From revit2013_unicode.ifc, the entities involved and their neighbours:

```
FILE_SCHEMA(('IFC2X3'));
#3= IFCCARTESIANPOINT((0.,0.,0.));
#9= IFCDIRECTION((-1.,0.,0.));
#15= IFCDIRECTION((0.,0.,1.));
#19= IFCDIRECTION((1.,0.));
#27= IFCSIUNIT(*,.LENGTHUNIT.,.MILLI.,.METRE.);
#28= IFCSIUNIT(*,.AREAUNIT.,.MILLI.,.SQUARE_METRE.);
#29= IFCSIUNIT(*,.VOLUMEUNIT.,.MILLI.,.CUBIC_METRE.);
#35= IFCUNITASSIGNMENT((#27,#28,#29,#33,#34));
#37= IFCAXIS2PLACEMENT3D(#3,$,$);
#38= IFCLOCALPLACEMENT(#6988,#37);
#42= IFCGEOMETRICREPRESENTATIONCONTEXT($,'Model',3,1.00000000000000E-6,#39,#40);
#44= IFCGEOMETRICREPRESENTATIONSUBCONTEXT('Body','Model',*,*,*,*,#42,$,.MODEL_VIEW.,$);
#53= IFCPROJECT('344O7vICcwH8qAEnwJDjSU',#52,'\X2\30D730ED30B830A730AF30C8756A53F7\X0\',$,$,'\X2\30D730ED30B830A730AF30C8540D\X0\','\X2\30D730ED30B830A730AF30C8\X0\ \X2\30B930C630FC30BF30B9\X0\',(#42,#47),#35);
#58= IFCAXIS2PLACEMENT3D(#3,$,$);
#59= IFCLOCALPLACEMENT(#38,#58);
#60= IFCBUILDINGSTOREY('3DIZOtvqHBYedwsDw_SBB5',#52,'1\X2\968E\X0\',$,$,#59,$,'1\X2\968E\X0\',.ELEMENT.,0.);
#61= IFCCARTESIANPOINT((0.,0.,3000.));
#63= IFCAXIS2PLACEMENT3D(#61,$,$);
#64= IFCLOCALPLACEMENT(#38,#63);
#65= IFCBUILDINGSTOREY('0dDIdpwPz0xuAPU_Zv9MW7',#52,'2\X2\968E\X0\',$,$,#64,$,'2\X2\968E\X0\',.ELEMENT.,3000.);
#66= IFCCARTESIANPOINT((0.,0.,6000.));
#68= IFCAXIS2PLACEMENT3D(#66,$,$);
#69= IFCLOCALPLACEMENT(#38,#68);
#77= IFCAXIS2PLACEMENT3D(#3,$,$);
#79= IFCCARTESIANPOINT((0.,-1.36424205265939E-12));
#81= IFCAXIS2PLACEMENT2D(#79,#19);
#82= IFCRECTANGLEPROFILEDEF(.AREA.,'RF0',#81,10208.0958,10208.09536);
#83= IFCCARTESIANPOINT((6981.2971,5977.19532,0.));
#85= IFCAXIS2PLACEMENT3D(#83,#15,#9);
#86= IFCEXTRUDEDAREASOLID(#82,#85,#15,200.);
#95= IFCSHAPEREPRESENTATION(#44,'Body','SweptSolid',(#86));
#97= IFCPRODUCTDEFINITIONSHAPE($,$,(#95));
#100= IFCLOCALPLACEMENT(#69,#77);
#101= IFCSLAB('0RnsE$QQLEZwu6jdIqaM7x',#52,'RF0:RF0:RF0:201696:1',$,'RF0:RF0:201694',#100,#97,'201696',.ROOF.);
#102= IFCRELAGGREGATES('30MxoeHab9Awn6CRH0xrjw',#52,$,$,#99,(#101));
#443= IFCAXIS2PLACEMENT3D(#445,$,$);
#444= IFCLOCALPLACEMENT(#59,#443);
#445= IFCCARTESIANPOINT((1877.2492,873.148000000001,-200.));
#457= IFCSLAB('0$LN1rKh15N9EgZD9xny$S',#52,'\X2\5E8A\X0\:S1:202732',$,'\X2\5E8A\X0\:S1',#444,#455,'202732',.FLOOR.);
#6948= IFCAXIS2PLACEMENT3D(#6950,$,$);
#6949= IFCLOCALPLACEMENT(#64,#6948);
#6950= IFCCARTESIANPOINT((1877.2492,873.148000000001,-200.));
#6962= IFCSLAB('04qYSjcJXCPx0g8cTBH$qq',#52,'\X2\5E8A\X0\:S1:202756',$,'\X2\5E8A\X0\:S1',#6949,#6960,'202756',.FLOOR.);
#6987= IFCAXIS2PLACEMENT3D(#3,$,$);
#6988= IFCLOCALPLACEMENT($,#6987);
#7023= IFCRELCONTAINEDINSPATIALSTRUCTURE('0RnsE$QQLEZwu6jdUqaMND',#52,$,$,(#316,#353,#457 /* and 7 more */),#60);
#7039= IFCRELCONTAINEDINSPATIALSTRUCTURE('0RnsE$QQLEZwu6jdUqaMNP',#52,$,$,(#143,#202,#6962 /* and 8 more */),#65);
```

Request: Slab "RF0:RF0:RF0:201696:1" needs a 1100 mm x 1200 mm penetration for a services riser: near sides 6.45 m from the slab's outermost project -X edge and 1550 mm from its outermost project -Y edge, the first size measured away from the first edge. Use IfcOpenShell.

```python
import numpy as np
import ifcopenshell
import ifcopenshell.api.feature
import ifcopenshell.api.geometry
import ifcopenshell.api.root
import ifcopenshell.geom
import ifcopenshell.util.placement
import ifcopenshell.util.representation
import ifcopenshell.util.shape
import ifcopenshell.util.unit

model = ifcopenshell.open("revit2013_unicode.ifc")
unit_scale = ifcopenshell.util.unit.calculate_unit_scale(model)
settings = ifcopenshell.geom.settings()


def volume(element):
    """Net volume in cubic metres, openings subtracted."""
    shape = ifcopenshell.geom.create_shape(settings, element)
    return ifcopenshell.util.shape.get_volume(shape.geometry)


slab = model.by_guid("0RnsE$QQLEZwu6jdIqaM7x")
before = volume(slab)

# Extent in the slab's own axes, in metres. The edges named are its -X and -Y sides.
slab_shape = ifcopenshell.geom.create_shape(settings, slab)
vertices = ifcopenshell.util.shape.get_vertices(slab_shape.geometry)
x_min, y_min, bottom = vertices.min(axis=0)
top = vertices[:, 2].max()

opening = ifcopenshell.api.root.create_entity(model, ifc_class="IfcOpeningElement", name="Services riser opening")
context = ifcopenshell.util.representation.get_context(model, "Model", "Body", "MODEL_VIEW")
width, depth = 1.1, 1.2
outline = [(0.0, 0.0), (width, 0.0), (width, depth), (0.0, depth), (0.0, 0.0)]
# Overshoot both faces by 50 mm so the cut is clean.
shape = ifcopenshell.api.geometry.add_slab_representation(
    model, context=context, depth=top - bottom + 0.1, polyline=outline
)
ifcopenshell.api.geometry.assign_representation(model, product=opening, representation=shape)

matrix = ifcopenshell.util.placement.get_local_placement(slab.ObjectPlacement)
matrix[:, 3] = matrix @ np.append(np.array([x_min + 6.45, y_min + 1.55, bottom - 0.05]) / unit_scale, 1.0)
ifcopenshell.api.geometry.edit_object_placement(model, product=opening, matrix=matrix, is_si=False)
ifcopenshell.api.feature.add_feature(model, feature=opening, element=slab)

after = volume(slab)

print(f"slab volume {before:.3f} -> {after:.3f} m3")

model.write("revit2013_unicode-out.ifc")
```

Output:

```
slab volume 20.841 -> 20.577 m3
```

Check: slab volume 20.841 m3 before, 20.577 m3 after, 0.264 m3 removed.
